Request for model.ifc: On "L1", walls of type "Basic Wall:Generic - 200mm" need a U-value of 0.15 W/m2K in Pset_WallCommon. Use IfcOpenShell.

First a look at what the model holds.

```python
import ifcopenshell
import ifcopenshell.util.element

model = ifcopenshell.open("model.ifc")
print(model.schema)
storey = next(s for s in model.by_type("IfcBuildingStorey") if s.Name == "L1")
walls = [e for e in ifcopenshell.util.element.get_decomposition(storey) if e.is_a("IfcWall")]
seen = {}
for e in walls:
    element_type = ifcopenshell.util.element.get_type(e)
    key = (element_type.Name if element_type != e and element_type else None, ifcopenshell.util.element.get_pset(e, "Pset_WallCommon", "ThermalTransmittance"))
    seen[key] = seen.get(key, 0) + 1
for (name, value), count in sorted(seen.items(), key=str):
    print(count, "x", name, "|", value)
```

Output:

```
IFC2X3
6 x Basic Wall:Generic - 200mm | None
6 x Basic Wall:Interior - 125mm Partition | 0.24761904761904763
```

```python
import ifcopenshell
import ifcopenshell.api.pset
import ifcopenshell.util.element

model = ifcopenshell.open("model.ifc")

storey = next(s for s in model.by_type("IfcBuildingStorey") if s.Name == "L1")
walls = [e for e in ifcopenshell.util.element.get_decomposition(storey) if e.is_a("IfcWall")]

count = 0
for e in walls:
    element_type = ifcopenshell.util.element.get_type(e)
    if element_type in (None, e) or element_type.Name != "Basic Wall:Generic - 200mm":
        continue
    # add_pset returns the element's existing set when there is one.
    pset = ifcopenshell.api.pset.add_pset(model, product=e, name="Pset_WallCommon")
    ifcopenshell.api.pset.edit_pset(model, pset=pset, properties={"ThermalTransmittance": 0.15})
    count += 1

print(count, "walls updated")

model.write("model_edited.ifc")
```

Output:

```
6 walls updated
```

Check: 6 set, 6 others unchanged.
